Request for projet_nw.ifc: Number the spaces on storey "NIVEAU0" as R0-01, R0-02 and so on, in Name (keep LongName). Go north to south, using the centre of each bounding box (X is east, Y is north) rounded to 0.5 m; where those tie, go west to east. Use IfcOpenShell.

First a look at what the model holds.

```python
import ifcopenshell
import ifcopenshell.util.element
import ifcopenshell.util.placement

model = ifcopenshell.open("projet_nw.ifc")
print(model.schema)
storey = next(s for s in model.by_type("IfcBuildingStorey") if s.Name == "NIVEAU0")
spaces = [e for e in ifcopenshell.util.element.get_decomposition(storey) if e.is_a("IfcSpace")]
for e in sorted(spaces, key=lambda e: e.id()):
    origin = ifcopenshell.util.placement.get_local_placement(e.ObjectPlacement)[:3, 3]
    print(e.id(), e.Name, e.LongName, origin.round(2) + 0.0, sep=" | ")
```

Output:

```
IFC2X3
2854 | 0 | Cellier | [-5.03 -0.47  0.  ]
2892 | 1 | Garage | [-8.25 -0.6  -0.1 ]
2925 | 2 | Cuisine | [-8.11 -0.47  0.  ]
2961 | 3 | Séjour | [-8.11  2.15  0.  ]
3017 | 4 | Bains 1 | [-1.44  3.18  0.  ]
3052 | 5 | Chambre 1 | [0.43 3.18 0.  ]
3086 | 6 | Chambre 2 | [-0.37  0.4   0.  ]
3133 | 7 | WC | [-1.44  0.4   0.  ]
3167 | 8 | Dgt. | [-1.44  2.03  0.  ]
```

```python
import ifcopenshell
import ifcopenshell.geom
import ifcopenshell.util.element
import ifcopenshell.util.shape

model = ifcopenshell.open("projet_nw.ifc")
settings = ifcopenshell.geom.settings()
settings.set("use-world-coords", True)


def centre(element):
    shape = ifcopenshell.geom.create_shape(settings, element)
    return ifcopenshell.util.shape.get_bbox_centroid(shape.geometry)


storey = next(s for s in model.by_type("IfcBuildingStorey") if s.Name == "NIVEAU0")
spaces = [e for e in ifcopenshell.util.element.get_decomposition(storey) if e.is_a("IfcSpace")]

# Insertion points can sit at a corner or the storey origin, so sort by the geometry (in metres).
centres = {e: centre(e) for e in spaces}
spaces.sort(key=lambda e: (-round(centres[e][1] / 0.5), centres[e][0]))

for i, e in enumerate(spaces, start=1):
    number = f"R0-{i:02d}"
    e.Name = number
    print(e.id(), number)

model.write("projet_nw-out.ifc")
```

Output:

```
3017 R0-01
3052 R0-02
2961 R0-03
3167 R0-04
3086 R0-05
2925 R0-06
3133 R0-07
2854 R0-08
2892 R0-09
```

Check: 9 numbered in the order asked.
